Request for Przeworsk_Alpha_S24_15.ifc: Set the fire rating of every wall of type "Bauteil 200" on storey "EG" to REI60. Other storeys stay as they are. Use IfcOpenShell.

First a look at what the model holds.

```python
import ifcopenshell
import ifcopenshell.util.element

model = ifcopenshell.open("Przeworsk_Alpha_S24_15.ifc")
print(model.schema)
storey = next(s for s in model.by_type("IfcBuildingStorey") if s.Name == "EG")
walls = [e for e in ifcopenshell.util.element.get_decomposition(storey) if e.is_a("IfcWall")]
seen = {}
for e in walls:
    element_type = ifcopenshell.util.element.get_type(e)
    key = (element_type.Name if element_type != e and element_type else None, ifcopenshell.util.element.get_pset(e, "Pset_WallCommon", "FireRating"))
    seen[key] = seen.get(key, 0) + 1
for (name, value), count in sorted(seen.items(), key=str):
    print(count, "x", name, "|", value)
```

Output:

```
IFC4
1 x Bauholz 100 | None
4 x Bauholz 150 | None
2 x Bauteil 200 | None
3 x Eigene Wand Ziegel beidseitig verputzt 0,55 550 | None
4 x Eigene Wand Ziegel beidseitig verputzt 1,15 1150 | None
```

```python
import ifcopenshell
import ifcopenshell.api.pset
import ifcopenshell.util.element

model = ifcopenshell.open("Przeworsk_Alpha_S24_15.ifc")

storey = next(s for s in model.by_type("IfcBuildingStorey") if s.Name == "EG")
walls = [e for e in ifcopenshell.util.element.get_decomposition(storey) if e.is_a("IfcWall")]

count = 0
for e in walls:
    element_type = ifcopenshell.util.element.get_type(e)
    if element_type in (None, e) or element_type.Name != "Bauteil 200":
        continue
    # add_pset returns the element's existing set when there is one.
    pset = ifcopenshell.api.pset.add_pset(model, product=e, name="Pset_WallCommon")
    ifcopenshell.api.pset.edit_pset(model, pset=pset, properties={"FireRating": "REI60"})
    count += 1

print(count, "walls updated")

model.write("Przeworsk_Alpha_S24_15-out.ifc")
```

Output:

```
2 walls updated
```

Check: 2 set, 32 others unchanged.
